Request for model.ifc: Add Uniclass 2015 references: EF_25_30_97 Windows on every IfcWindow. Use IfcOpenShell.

First a look at what the model holds.

```python
import ifcopenshell

model = ifcopenshell.open("model.ifc")
print(model.schema)
print("classifications:", [c.Name for c in model.by_type("IfcClassification")])
for ifc_class in ("IfcDoor", "IfcRoof", "IfcStair", "IfcWall", "IfcWindow"):
    print(ifc_class, len(model.by_type(ifc_class)))
```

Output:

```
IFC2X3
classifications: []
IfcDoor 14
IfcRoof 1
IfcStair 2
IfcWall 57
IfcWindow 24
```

```python
import ifcopenshell
import ifcopenshell.api.classification

model = ifcopenshell.open("model.ifc")

# IFC2X3 requires Source and Edition and has no link from the project to the system.
system = model.create_entity("IfcClassification", Source="NBS", Edition="2015", Name="Uniclass 2015")

codes = {
    "IfcWindow": ("EF_25_30_97", "Windows"),
}
for ifc_class, (code, name) in codes.items():
    products = model.by_type(ifc_class)
    ifcopenshell.api.classification.add_reference(
        model, products=products, classification=system, identification=code, name=name
    )
    print(code, len(products))

model.write("model_rev.ifc")
```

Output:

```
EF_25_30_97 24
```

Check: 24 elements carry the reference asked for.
